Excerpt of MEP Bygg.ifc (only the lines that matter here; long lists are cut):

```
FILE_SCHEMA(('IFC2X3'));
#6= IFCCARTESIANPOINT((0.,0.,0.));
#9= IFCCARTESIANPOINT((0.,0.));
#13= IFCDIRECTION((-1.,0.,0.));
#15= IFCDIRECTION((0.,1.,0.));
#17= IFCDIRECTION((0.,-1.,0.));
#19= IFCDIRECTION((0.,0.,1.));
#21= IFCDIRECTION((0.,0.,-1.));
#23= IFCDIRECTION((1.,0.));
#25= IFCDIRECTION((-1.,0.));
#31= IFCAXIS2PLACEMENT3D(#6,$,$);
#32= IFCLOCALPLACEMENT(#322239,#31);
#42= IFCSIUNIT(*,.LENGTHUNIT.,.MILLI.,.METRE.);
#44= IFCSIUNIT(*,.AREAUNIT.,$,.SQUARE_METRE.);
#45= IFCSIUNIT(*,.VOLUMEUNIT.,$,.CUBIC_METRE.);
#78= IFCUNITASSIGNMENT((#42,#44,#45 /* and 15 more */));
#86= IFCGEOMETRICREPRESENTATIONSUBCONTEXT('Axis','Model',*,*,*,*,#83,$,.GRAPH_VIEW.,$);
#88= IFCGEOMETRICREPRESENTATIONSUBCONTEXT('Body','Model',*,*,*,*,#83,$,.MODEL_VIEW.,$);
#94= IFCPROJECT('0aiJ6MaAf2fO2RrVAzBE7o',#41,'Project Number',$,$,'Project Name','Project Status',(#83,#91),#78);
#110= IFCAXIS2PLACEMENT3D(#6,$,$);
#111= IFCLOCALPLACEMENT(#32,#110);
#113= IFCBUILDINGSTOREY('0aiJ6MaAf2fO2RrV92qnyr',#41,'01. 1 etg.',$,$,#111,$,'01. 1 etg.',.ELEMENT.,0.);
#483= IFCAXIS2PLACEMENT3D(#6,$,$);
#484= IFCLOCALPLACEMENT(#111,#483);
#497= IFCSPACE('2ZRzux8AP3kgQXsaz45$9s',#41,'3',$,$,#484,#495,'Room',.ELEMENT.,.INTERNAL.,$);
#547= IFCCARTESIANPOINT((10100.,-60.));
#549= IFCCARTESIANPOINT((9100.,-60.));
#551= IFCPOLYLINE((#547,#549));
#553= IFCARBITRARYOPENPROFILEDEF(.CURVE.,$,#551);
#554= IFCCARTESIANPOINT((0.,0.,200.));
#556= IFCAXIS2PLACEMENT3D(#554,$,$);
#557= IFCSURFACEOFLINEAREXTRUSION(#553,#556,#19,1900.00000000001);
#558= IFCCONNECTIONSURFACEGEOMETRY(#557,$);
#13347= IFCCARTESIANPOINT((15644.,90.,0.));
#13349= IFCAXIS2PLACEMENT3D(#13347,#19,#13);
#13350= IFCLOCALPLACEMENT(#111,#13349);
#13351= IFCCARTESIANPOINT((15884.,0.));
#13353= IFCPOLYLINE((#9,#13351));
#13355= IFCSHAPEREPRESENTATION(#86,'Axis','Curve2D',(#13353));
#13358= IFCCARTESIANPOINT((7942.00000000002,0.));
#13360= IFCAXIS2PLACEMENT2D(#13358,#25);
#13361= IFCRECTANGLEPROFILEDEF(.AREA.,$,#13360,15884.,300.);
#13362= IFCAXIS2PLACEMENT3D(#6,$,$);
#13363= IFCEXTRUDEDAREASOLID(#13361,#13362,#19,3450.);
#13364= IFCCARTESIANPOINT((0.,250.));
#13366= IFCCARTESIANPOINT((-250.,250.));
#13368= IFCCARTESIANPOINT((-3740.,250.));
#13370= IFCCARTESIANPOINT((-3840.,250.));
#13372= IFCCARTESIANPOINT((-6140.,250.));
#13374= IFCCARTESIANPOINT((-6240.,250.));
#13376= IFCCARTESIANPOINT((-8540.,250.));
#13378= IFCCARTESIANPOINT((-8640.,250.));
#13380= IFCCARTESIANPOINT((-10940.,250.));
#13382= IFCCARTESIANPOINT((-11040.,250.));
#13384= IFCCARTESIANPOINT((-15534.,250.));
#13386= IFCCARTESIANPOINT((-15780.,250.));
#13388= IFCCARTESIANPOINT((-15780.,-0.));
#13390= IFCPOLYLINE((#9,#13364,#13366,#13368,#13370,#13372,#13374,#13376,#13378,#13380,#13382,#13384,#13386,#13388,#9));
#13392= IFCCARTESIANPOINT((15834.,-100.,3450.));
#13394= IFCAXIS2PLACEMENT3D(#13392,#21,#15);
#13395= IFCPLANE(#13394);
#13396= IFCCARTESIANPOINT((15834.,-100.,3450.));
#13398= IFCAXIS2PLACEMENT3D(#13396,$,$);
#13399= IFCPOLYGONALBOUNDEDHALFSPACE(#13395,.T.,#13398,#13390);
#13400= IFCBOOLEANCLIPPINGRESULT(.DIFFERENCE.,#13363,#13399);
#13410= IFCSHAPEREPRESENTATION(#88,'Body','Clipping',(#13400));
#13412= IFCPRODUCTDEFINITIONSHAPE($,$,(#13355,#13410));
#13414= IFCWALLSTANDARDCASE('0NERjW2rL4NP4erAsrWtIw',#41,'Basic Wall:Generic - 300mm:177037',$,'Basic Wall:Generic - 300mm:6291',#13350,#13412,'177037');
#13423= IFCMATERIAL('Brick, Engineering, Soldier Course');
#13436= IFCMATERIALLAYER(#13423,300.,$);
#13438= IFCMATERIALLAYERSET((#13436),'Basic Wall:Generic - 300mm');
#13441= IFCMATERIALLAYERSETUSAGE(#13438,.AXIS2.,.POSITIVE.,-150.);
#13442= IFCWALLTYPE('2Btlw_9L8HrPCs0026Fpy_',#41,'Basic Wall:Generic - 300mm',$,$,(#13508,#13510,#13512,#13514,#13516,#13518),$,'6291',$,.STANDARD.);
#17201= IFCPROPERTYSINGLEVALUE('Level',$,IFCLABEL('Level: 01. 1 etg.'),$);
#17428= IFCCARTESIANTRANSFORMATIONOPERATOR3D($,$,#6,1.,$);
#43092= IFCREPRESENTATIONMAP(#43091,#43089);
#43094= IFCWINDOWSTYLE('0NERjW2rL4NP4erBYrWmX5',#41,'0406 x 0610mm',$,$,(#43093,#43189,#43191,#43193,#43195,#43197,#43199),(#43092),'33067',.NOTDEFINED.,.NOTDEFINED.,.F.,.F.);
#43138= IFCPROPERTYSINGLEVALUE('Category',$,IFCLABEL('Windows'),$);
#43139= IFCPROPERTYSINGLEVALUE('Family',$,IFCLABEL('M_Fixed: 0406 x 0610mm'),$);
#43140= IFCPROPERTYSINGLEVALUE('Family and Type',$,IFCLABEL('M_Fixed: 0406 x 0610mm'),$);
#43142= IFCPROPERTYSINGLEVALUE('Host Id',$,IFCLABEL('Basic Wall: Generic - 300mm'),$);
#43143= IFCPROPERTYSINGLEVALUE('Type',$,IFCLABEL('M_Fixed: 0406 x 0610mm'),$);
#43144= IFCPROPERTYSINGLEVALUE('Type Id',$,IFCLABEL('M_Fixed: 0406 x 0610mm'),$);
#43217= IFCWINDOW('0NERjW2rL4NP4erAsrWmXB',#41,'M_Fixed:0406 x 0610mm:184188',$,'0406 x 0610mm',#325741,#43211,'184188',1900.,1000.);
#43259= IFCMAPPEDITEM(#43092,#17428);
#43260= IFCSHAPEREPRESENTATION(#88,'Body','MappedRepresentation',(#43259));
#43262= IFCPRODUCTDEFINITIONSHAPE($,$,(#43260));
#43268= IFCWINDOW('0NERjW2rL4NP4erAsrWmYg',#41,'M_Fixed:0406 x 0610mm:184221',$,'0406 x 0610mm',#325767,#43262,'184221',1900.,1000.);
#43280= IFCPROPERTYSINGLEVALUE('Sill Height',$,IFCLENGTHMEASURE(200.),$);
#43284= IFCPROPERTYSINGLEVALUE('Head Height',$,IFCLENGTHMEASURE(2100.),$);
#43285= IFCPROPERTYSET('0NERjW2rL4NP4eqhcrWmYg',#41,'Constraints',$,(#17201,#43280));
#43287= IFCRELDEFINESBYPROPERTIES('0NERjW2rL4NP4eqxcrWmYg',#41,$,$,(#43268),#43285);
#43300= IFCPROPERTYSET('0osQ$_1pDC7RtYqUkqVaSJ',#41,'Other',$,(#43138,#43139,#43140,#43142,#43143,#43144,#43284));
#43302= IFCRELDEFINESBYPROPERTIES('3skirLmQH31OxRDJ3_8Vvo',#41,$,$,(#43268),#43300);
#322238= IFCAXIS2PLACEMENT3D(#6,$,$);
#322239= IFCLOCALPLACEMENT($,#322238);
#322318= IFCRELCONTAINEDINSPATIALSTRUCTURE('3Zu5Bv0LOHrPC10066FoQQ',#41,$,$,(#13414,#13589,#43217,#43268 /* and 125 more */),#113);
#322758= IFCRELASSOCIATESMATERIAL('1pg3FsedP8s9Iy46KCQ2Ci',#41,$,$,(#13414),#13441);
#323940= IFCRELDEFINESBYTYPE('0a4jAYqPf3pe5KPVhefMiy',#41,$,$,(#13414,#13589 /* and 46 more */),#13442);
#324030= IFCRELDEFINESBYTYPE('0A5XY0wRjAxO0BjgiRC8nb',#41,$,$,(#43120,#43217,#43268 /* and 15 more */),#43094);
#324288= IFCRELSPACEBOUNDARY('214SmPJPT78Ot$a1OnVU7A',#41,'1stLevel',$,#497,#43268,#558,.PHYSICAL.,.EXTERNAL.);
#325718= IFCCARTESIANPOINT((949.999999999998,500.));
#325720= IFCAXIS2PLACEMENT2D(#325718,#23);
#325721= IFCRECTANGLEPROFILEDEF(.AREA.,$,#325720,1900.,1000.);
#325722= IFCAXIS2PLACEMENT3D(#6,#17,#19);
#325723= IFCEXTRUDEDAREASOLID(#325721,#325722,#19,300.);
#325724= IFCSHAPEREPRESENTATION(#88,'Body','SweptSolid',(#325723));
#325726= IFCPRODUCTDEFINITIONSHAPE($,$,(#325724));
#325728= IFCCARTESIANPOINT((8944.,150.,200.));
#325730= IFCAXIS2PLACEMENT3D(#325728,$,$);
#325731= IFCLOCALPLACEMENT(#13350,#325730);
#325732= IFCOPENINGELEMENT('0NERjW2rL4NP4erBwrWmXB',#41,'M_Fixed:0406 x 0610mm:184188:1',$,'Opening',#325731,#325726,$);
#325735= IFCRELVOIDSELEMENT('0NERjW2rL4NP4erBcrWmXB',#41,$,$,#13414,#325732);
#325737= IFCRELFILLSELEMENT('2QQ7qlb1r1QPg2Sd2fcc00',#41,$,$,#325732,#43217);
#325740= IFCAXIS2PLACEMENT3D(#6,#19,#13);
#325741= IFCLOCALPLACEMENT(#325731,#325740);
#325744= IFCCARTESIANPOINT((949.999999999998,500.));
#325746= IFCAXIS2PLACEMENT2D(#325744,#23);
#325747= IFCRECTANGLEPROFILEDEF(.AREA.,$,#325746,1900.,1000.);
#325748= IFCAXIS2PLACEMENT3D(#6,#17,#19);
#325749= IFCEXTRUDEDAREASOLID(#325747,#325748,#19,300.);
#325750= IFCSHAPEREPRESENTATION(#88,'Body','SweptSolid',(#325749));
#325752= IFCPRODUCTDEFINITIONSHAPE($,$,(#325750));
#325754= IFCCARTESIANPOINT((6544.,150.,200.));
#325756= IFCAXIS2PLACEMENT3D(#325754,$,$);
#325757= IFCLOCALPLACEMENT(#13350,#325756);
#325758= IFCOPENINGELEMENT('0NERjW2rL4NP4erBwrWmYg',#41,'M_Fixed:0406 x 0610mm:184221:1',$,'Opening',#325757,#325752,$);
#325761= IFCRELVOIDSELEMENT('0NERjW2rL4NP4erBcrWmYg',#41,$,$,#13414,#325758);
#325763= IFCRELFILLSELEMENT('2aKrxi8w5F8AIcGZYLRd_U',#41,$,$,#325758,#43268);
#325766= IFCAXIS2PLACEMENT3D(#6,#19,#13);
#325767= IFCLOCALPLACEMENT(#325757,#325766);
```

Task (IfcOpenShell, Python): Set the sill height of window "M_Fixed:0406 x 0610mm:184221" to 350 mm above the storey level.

```python
import numpy as np
import ifcopenshell
import ifcopenshell.api.geometry
import ifcopenshell.api.pset
import ifcopenshell.geom
import ifcopenshell.util.element
import ifcopenshell.util.placement
import ifcopenshell.util.shape
import ifcopenshell.util.unit

model = ifcopenshell.open("MEP Bygg.ifc")
unit_scale = ifcopenshell.util.unit.calculate_unit_scale(model)

window = model.by_guid("0NERjW2rL4NP4erAsrWmYg")
opening = window.FillsVoids[0].RelatingOpeningElement
storey = ifcopenshell.util.element.get_container(window, ifc_class="IfcBuildingStorey")
level = ifcopenshell.util.placement.get_local_placement(storey.ObjectPlacement)[2, 3]

# The opening's origin need not be at the sill, so measure its lowest point.
shape = ifcopenshell.geom.create_shape(ifcopenshell.geom.settings(), opening)
bottom = ifcopenshell.util.shape.get_shape_bottom_elevation(shape, shape.geometry) / unit_scale
dz = level + 350.0 - bottom

shift = np.array([0.0, 0.0, dz])
# The window is placed relative to its opening, so it follows when the opening moves.
matrix = ifcopenshell.util.placement.get_local_placement(opening.ObjectPlacement)
matrix[:3, 3] += shift
ifcopenshell.api.geometry.edit_object_placement(
    model, product=opening, matrix=matrix, is_si=False, should_transform_children=True
)

# Space boundary surfaces are stored in each space's coordinates; move them too.
for rel in window.ProvidesBoundaries:
    if not rel.ConnectionGeometry:
        continue
    surface = rel.ConnectionGeometry.SurfaceOnRelatingElement
    space_matrix = ifcopenshell.util.placement.get_local_placement(rel.RelatingSpace.ObjectPlacement)
    point = np.array(surface.Position.Location.Coordinates) + space_matrix[:3, :3].T @ shift
    surface.Position = model.createIfcAxis2Placement3D(
        model.createIfcCartesianPoint(point.tolist()), surface.Position.Axis, surface.Position.RefDirection
    )

# Keep the stored heights in step.
pset = model.by_id(ifcopenshell.util.element.get_pset(window, "Constraints", should_inherit=False)["id"])
ifcopenshell.api.pset.edit_pset(model, pset=pset, properties={
    "Sill Height": model.create_entity("IfcLengthMeasure", ifcopenshell.util.element.get_pset(window, "Constraints", "Sill Height") + dz),
})
pset = model.by_id(ifcopenshell.util.element.get_pset(window, "Other", should_inherit=False)["id"])
ifcopenshell.api.pset.edit_pset(model, pset=pset, properties={
    "Head Height": model.create_entity("IfcLengthMeasure", ifcopenshell.util.element.get_pset(window, "Other", "Head Height") + dz),
})

print(f"moved by {dz * unit_scale:+.3f} m")

model.write("MEP Bygg_v2.ifc")
```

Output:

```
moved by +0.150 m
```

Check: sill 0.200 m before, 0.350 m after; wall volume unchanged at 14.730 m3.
